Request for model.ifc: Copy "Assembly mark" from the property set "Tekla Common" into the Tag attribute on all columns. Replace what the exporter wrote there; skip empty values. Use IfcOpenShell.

First a look at what the model holds.

```python
import ifcopenshell
import ifcopenshell.util.element

model = ifcopenshell.open("model.ifc")
print(model.schema)
columns = model.by_type("IfcColumn")
print(len(columns), "columns")
for e in columns[:8]:
    source = ifcopenshell.util.element.get_pset(e, "Tekla Common", "Assembly mark")
    target = e.Tag
    print(e.id(), repr(source), repr(target), sep=" | ")
```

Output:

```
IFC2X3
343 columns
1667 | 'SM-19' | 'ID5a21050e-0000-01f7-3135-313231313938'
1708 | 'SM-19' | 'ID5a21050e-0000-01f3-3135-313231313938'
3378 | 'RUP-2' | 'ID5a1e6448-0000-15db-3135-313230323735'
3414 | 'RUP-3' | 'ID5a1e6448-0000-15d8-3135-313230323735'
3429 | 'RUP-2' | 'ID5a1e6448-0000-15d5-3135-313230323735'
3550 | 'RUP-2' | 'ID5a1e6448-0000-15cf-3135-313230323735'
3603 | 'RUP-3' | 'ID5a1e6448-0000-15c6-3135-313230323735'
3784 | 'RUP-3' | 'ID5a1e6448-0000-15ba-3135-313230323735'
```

```python
import ifcopenshell
import ifcopenshell.util.element

model = ifcopenshell.open("model.ifc")

count = 0
for e in model.by_type("IfcColumn"):
    value = ifcopenshell.util.element.get_pset(e, "Tekla Common", "Assembly mark")
    current = e.Tag
    if not value or not value.strip() or current == value:
        continue
    e.Tag = value
    count += 1

print(count, "columns updated")

model.write("model_v2.ifc")
```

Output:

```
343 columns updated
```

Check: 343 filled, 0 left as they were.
